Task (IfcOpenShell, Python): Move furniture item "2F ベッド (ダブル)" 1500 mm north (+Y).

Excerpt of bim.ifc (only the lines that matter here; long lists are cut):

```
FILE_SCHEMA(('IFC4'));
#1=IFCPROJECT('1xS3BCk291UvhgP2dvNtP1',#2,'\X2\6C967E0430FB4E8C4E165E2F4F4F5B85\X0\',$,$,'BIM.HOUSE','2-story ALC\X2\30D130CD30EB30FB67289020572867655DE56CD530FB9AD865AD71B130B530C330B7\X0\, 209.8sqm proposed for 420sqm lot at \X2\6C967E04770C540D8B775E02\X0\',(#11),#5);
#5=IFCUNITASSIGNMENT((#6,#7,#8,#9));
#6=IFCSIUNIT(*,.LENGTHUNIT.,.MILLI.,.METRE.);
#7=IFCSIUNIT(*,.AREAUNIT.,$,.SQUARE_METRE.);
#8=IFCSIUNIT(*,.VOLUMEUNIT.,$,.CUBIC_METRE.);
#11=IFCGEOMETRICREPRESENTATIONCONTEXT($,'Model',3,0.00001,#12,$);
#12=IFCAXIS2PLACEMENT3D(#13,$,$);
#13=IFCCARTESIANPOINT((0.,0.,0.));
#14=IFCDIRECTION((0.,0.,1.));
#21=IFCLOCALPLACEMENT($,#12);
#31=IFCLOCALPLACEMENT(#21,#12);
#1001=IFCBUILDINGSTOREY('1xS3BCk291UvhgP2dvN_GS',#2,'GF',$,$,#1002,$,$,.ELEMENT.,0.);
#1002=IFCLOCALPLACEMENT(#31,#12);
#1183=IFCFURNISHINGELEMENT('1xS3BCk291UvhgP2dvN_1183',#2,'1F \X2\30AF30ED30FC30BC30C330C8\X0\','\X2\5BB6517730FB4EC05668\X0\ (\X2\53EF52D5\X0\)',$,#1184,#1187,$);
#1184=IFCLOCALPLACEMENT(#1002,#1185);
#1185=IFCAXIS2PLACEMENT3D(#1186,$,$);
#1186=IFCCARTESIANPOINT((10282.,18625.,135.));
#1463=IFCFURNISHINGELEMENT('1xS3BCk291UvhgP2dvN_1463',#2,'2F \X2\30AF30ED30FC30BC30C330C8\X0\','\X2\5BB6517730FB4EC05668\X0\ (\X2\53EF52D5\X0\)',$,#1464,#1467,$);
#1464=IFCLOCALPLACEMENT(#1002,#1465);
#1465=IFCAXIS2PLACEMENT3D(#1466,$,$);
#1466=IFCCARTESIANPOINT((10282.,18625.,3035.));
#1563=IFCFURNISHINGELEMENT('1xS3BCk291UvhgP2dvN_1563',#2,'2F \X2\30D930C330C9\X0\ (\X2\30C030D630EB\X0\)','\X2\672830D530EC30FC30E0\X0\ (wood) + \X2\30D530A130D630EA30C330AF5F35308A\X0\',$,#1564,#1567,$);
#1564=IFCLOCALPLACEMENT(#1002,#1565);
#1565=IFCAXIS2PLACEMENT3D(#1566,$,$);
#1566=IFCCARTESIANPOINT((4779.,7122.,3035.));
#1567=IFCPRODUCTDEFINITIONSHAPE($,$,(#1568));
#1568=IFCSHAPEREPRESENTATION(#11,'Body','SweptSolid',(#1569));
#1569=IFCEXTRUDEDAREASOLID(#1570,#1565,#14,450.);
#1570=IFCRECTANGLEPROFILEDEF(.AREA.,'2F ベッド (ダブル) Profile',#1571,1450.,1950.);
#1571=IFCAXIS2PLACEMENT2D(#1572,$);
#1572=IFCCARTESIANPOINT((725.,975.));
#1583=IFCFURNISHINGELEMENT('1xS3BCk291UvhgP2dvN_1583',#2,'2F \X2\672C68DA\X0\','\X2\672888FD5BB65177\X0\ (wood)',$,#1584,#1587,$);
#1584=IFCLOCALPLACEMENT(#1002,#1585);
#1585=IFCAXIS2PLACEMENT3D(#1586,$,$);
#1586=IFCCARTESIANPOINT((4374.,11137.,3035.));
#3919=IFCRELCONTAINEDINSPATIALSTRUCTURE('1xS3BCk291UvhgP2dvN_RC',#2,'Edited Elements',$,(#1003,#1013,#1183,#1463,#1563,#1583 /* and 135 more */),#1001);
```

```python
import ifcopenshell
import ifcopenshell.api.geometry
import ifcopenshell.util.placement
import ifcopenshell.util.unit

model = ifcopenshell.open("bim.ifc")
unit_scale = ifcopenshell.util.unit.calculate_unit_scale(model)

item = model.by_id(1563)
matrix = ifcopenshell.util.placement.get_local_placement(item.ObjectPlacement)
matrix[1, 3] += 1.5 / unit_scale
ifcopenshell.api.geometry.edit_object_placement(model, product=item, matrix=matrix, is_si=False)

print(ifcopenshell.util.placement.get_local_placement(item.ObjectPlacement).round(3) + 0.0)

model.write("bim_updated.ifc")
```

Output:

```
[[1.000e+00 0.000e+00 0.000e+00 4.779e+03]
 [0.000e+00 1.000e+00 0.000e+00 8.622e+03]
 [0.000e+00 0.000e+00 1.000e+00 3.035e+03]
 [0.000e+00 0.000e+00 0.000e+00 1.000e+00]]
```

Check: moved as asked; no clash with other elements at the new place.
